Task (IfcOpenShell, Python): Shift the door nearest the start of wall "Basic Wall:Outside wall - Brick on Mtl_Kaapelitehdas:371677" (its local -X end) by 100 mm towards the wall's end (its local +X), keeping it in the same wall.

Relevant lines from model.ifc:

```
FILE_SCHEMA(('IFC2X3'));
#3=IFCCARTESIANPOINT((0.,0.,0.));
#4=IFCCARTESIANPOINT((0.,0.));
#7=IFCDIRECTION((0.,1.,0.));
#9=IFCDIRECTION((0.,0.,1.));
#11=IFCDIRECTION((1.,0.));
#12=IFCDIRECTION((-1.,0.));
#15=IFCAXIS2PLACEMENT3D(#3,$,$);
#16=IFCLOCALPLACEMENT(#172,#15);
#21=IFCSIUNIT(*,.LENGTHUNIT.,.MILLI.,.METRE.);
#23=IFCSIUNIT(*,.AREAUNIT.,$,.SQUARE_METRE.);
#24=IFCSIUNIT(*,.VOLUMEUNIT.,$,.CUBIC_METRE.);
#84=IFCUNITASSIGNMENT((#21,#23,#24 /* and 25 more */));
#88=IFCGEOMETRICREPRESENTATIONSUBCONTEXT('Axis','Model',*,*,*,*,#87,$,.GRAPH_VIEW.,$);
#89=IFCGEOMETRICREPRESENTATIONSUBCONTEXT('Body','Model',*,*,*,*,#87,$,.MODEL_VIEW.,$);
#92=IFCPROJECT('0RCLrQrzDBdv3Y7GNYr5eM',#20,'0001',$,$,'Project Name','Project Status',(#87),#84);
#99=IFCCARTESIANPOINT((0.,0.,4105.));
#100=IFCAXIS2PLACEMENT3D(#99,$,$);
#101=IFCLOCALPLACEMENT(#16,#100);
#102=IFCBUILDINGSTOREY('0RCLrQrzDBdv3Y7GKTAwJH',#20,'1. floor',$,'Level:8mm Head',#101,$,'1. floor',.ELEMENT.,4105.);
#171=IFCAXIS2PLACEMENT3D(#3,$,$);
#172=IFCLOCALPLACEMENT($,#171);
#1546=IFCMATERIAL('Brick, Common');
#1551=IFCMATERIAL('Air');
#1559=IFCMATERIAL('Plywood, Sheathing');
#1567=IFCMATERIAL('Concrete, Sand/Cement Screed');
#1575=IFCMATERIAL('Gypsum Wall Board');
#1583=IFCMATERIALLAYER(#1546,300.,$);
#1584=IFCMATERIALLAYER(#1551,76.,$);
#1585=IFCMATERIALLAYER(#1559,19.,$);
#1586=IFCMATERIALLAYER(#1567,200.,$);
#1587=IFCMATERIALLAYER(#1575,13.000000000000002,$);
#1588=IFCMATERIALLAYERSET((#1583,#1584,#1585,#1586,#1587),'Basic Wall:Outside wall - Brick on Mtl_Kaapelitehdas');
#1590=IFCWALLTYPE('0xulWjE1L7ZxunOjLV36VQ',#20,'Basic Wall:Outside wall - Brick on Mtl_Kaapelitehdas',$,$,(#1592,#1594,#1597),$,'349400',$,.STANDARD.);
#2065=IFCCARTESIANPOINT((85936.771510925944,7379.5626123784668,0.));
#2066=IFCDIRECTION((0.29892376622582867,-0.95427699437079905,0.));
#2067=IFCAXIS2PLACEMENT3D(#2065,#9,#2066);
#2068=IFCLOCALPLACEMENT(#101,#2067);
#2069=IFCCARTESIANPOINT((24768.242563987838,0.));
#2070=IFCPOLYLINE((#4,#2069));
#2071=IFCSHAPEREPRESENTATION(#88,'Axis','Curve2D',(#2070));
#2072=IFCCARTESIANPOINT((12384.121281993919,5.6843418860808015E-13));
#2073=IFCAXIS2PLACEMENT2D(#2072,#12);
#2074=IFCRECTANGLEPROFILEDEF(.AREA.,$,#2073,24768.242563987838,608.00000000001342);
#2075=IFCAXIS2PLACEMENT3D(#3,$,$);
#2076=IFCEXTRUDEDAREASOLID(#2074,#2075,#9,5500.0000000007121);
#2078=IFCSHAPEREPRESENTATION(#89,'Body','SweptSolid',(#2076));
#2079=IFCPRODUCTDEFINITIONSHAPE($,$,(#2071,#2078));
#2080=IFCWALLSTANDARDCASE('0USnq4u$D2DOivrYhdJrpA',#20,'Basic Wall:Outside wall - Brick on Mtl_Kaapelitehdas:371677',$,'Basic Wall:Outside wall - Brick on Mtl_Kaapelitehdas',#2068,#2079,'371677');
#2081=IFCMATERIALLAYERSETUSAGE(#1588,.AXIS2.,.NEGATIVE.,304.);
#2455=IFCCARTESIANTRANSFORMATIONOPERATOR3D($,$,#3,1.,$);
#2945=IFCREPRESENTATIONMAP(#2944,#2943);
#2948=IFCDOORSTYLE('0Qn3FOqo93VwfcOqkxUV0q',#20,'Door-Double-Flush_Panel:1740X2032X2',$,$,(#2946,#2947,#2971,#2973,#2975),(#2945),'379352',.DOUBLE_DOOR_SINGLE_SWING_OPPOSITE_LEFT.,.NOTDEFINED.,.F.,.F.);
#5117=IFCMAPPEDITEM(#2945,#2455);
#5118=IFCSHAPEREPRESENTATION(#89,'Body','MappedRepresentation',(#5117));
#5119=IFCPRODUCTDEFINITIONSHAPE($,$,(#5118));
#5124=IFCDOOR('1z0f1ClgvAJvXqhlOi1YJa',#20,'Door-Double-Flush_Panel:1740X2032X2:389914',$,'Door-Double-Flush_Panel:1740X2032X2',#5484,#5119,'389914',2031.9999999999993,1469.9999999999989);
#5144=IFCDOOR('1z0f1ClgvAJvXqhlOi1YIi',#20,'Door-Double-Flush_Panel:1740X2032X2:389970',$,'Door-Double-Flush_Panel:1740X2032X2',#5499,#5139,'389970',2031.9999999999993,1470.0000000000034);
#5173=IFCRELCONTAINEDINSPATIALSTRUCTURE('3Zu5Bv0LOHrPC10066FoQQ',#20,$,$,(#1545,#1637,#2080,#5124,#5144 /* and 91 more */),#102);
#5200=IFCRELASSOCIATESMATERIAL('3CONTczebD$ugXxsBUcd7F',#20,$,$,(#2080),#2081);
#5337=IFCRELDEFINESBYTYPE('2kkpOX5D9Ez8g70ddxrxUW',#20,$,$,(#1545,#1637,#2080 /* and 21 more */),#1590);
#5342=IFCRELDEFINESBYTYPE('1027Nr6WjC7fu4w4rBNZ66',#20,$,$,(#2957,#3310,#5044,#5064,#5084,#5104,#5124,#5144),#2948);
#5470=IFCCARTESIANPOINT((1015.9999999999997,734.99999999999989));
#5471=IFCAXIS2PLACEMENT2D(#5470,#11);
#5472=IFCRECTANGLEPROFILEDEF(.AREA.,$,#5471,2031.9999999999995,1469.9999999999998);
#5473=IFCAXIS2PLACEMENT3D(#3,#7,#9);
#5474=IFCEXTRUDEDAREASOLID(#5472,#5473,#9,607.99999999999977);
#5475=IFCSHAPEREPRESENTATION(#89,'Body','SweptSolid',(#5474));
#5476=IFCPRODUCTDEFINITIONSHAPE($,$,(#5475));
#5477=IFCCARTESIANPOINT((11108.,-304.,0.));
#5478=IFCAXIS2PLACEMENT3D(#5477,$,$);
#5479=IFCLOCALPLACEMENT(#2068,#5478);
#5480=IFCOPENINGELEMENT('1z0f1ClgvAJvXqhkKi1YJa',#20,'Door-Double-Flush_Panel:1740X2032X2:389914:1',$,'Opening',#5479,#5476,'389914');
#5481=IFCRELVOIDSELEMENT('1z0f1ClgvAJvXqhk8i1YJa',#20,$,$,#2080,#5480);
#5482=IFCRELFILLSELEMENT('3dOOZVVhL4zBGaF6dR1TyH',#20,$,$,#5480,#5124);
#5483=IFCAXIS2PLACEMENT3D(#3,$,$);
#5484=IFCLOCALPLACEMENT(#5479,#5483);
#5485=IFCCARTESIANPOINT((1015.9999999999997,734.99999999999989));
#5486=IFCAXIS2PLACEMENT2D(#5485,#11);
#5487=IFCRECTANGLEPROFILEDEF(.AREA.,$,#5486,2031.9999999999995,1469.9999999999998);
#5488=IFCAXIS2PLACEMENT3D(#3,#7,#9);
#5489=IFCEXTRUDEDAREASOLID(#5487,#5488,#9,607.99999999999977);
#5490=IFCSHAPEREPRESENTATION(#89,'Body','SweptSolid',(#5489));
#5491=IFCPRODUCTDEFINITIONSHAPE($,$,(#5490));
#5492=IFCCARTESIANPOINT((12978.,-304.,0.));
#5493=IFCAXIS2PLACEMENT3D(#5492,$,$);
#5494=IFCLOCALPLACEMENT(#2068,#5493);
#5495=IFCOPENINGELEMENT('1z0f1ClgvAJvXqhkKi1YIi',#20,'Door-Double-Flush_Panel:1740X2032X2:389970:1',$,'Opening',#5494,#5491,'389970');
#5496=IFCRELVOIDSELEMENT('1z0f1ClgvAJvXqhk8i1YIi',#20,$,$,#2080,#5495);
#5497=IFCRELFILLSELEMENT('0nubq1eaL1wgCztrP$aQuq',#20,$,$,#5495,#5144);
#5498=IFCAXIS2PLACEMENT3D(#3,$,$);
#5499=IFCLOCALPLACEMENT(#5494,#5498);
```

```python
import ifcopenshell
import ifcopenshell.api.geometry
import ifcopenshell.util.placement

model = ifcopenshell.open("model.ifc")

door = model.by_guid("1z0f1ClgvAJvXqhlOi1YJa")
opening = door.FillsVoids[0].RelatingOpeningElement
wall = opening.VoidsElements[0].RelatingBuildingElement

wall_matrix = ifcopenshell.util.placement.get_local_placement(wall.ObjectPlacement)
shift = wall_matrix[:3, 0] * 100.0
before = ifcopenshell.util.placement.get_local_placement(door.ObjectPlacement)[:3, 3].copy()

# The door is placed relative to its opening, so it follows when the opening moves.
matrix = ifcopenshell.util.placement.get_local_placement(opening.ObjectPlacement)
matrix[:3, 3] += shift
ifcopenshell.api.geometry.edit_object_placement(
    model, product=opening, matrix=matrix, is_si=False, should_transform_children=True
)

after = ifcopenshell.util.placement.get_local_placement(door.ObjectPlacement)[:3, 3]
print("door moved by", (after - before).round(3) + 0.0)

model.write("model-out.ifc")
```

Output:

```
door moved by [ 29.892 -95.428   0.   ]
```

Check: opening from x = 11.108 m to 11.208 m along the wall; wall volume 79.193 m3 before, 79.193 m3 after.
